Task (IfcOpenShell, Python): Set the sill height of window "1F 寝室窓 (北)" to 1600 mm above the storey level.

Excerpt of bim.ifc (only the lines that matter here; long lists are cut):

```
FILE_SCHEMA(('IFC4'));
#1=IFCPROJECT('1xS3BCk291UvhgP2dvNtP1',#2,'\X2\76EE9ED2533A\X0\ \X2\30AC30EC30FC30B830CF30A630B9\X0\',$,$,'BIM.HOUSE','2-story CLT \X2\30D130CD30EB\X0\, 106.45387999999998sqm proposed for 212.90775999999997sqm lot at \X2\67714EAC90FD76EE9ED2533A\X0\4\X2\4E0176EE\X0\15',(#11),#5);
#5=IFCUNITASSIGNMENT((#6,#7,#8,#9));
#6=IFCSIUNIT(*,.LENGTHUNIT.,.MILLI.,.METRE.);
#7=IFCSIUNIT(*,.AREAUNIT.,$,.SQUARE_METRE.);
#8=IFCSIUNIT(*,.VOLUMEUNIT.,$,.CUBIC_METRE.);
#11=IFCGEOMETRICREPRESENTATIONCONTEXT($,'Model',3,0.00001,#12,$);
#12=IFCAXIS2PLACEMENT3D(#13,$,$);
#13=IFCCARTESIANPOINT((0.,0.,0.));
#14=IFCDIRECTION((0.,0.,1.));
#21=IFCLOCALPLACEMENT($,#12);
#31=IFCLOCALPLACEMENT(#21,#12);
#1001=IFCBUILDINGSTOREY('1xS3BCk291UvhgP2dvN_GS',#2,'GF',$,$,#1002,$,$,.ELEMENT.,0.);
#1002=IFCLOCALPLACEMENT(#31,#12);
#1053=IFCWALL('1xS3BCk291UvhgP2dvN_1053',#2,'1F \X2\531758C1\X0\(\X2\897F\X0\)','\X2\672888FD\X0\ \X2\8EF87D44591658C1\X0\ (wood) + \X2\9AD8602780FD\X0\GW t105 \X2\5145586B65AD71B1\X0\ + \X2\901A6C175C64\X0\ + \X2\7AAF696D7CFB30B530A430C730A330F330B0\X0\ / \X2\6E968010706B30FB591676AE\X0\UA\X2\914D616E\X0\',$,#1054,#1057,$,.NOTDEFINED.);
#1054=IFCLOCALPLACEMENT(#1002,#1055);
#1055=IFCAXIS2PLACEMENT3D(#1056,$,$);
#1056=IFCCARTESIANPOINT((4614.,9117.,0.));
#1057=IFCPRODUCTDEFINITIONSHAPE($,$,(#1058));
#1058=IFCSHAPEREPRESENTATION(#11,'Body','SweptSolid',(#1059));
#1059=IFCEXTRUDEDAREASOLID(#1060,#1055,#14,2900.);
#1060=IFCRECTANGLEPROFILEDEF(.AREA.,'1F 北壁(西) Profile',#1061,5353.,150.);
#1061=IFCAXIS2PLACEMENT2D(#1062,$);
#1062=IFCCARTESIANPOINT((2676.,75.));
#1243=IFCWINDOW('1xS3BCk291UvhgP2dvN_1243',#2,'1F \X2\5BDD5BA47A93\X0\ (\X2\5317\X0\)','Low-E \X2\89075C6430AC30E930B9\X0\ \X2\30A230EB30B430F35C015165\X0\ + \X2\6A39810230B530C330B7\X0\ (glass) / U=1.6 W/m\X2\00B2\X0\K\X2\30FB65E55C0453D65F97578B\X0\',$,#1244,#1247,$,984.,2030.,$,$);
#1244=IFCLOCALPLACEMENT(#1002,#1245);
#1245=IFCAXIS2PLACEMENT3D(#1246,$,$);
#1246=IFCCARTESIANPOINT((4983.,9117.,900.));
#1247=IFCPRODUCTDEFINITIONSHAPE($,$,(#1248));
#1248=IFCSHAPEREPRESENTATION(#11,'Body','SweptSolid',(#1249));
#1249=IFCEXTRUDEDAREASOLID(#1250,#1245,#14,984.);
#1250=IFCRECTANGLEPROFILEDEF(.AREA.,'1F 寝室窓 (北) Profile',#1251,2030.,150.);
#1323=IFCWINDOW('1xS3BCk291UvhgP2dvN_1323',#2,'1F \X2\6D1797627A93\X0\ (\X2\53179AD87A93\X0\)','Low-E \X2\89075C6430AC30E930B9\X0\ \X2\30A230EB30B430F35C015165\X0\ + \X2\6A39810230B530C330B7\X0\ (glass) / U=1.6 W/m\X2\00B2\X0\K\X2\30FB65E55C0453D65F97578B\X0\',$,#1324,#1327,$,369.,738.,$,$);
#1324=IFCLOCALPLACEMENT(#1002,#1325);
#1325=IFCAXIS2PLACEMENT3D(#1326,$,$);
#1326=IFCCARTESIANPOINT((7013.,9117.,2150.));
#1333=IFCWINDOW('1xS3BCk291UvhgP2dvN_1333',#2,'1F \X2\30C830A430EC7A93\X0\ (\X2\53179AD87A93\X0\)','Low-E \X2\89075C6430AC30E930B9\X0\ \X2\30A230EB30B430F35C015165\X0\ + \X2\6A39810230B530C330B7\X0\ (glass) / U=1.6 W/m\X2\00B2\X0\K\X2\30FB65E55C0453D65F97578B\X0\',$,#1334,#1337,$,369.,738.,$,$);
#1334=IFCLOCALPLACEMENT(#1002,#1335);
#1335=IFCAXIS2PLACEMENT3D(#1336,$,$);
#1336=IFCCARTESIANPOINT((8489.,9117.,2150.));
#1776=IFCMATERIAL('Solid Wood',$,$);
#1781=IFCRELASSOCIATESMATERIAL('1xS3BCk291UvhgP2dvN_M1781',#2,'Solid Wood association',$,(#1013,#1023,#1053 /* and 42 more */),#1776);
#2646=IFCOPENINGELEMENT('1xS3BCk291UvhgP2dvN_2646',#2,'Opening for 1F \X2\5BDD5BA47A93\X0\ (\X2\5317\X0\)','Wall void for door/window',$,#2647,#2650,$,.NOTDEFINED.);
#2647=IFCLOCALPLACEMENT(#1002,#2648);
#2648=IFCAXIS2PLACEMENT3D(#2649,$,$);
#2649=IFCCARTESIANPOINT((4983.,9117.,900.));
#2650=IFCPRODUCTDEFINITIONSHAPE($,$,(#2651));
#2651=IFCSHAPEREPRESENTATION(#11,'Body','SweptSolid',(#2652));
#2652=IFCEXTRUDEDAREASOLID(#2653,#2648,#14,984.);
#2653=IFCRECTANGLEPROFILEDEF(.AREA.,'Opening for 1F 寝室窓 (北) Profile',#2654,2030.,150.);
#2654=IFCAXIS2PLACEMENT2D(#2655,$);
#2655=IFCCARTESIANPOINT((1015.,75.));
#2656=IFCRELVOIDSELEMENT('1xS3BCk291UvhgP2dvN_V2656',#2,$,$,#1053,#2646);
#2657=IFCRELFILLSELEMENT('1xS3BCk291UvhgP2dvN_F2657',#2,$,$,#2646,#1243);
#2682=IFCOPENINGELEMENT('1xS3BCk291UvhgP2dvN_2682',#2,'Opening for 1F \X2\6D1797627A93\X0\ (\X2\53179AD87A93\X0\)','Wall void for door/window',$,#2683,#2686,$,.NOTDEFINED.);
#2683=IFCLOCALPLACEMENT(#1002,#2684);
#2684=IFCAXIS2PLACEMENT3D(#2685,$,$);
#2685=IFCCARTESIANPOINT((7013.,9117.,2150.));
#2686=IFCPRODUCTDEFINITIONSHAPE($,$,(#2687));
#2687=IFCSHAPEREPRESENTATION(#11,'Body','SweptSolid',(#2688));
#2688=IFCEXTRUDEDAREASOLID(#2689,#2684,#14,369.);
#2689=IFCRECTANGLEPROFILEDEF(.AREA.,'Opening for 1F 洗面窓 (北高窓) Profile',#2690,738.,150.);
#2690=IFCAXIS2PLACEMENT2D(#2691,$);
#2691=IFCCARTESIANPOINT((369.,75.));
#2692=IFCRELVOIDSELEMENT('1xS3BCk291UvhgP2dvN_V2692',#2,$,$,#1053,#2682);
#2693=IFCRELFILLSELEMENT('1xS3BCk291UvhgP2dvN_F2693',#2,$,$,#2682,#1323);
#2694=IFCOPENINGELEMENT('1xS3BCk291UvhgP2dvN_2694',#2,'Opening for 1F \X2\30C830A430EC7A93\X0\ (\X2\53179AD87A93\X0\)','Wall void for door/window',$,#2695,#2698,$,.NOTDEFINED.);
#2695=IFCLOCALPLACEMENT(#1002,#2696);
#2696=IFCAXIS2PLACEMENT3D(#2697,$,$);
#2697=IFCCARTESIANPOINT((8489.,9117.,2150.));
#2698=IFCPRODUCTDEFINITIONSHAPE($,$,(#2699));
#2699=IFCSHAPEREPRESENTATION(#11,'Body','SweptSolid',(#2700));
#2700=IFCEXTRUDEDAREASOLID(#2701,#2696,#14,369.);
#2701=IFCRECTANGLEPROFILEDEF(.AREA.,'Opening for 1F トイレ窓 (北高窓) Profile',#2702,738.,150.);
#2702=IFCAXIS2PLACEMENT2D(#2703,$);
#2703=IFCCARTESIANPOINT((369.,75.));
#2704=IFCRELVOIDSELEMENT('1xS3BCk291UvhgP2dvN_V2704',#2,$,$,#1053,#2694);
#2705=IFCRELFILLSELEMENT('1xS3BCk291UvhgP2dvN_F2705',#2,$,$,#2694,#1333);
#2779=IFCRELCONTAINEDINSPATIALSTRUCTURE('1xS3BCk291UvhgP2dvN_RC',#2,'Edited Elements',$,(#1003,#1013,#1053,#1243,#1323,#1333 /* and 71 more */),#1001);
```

```python
import numpy as np
import ifcopenshell
import ifcopenshell.api.geometry
import ifcopenshell.geom
import ifcopenshell.util.element
import ifcopenshell.util.placement
import ifcopenshell.util.shape
import ifcopenshell.util.unit

model = ifcopenshell.open("bim.ifc")
unit_scale = ifcopenshell.util.unit.calculate_unit_scale(model)

window = model.by_id(1243)
opening = window.FillsVoids[0].RelatingOpeningElement
storey = ifcopenshell.util.element.get_container(window, ifc_class="IfcBuildingStorey")
level = ifcopenshell.util.placement.get_local_placement(storey.ObjectPlacement)[2, 3]

# The opening's origin need not be at the sill, so measure its lowest point.
shape = ifcopenshell.geom.create_shape(ifcopenshell.geom.settings(), opening)
bottom = ifcopenshell.util.shape.get_shape_bottom_elevation(shape, shape.geometry) / unit_scale
dz = level + 1600.0 - bottom

shift = np.array([0.0, 0.0, dz])
# The window is not placed relative to its opening, so move both.
for product in (opening, window):
    matrix = ifcopenshell.util.placement.get_local_placement(product.ObjectPlacement)
    matrix[:3, 3] += shift
    ifcopenshell.api.geometry.edit_object_placement(model, product=product, matrix=matrix, is_si=False)

print(f"moved by {dz * unit_scale:+.3f} m")

model.write("bim_v2.ifc")
```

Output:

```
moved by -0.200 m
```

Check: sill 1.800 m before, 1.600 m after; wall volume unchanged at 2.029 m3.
